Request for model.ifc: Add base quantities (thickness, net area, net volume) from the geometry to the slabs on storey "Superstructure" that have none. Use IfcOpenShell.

First a look at what the model holds.

```python
import ifcopenshell
import ifcopenshell.util.element
import ifcopenshell.util.unit

model = ifcopenshell.open("model.ifc")
print(model.schema)
for unit_type in ("LENGTHUNIT", "AREAUNIT", "VOLUMEUNIT"):
    print(unit_type, ifcopenshell.util.unit.calculate_unit_scale(model, unit_type))
storey = next(s for s in model.by_type("IfcBuildingStorey") if s.Name == "Superstructure")
slabs = [e for e in ifcopenshell.util.element.get_decomposition(storey) if e.is_a("IfcSlab")]
for e in sorted(slabs, key=lambda e: e.id()):
    print(e.id(), e.is_a(), e.Name, list(ifcopenshell.util.element.get_psets(e, qtos_only=True)), sep=" | ")
```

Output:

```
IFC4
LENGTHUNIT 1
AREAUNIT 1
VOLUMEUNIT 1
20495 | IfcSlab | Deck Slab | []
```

```python
import ifcopenshell
import ifcopenshell.api.pset
import ifcopenshell.geom
import ifcopenshell.util.element
import ifcopenshell.util.shape
import ifcopenshell.util.unit

model = ifcopenshell.open("model.ifc")
unit_scale = ifcopenshell.util.unit.calculate_unit_scale(model)
area_scale = ifcopenshell.util.unit.calculate_unit_scale(model, "AREAUNIT")
volume_scale = ifcopenshell.util.unit.calculate_unit_scale(model, "VOLUMEUNIT")
settings = ifcopenshell.geom.settings()

storey = next(s for s in model.by_type("IfcBuildingStorey") if s.Name == "Superstructure")
slabs = [e for e in ifcopenshell.util.element.get_decomposition(storey) if e.is_a("IfcSlab")]

for e in sorted(slabs, key=lambda e: e.id()):
    if ifcopenshell.util.element.get_psets(e, qtos_only=True, should_inherit=False):
        continue
    # Geometry comes back in metres, in the element's own axes.
    shape = ifcopenshell.geom.create_shape(settings, e)
    values = {
        "Width": ifcopenshell.util.shape.get_z(shape.geometry) / unit_scale,
        "NetArea": ifcopenshell.util.shape.get_footprint_area(shape.geometry) / area_scale,
        "NetVolume": ifcopenshell.util.shape.get_volume(shape.geometry) / volume_scale,
    }
    qto = ifcopenshell.api.pset.add_qto(model, product=e, name="Qto_SlabBaseQuantities")
    ifcopenshell.api.pset.edit_qto(model, qto=qto, properties=values)
    print(e.id(), {k: round(v, 3) for k, v in values.items()})

model.write("model-out.ifc")
```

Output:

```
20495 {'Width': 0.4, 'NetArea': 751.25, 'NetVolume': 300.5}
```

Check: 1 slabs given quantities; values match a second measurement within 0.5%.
